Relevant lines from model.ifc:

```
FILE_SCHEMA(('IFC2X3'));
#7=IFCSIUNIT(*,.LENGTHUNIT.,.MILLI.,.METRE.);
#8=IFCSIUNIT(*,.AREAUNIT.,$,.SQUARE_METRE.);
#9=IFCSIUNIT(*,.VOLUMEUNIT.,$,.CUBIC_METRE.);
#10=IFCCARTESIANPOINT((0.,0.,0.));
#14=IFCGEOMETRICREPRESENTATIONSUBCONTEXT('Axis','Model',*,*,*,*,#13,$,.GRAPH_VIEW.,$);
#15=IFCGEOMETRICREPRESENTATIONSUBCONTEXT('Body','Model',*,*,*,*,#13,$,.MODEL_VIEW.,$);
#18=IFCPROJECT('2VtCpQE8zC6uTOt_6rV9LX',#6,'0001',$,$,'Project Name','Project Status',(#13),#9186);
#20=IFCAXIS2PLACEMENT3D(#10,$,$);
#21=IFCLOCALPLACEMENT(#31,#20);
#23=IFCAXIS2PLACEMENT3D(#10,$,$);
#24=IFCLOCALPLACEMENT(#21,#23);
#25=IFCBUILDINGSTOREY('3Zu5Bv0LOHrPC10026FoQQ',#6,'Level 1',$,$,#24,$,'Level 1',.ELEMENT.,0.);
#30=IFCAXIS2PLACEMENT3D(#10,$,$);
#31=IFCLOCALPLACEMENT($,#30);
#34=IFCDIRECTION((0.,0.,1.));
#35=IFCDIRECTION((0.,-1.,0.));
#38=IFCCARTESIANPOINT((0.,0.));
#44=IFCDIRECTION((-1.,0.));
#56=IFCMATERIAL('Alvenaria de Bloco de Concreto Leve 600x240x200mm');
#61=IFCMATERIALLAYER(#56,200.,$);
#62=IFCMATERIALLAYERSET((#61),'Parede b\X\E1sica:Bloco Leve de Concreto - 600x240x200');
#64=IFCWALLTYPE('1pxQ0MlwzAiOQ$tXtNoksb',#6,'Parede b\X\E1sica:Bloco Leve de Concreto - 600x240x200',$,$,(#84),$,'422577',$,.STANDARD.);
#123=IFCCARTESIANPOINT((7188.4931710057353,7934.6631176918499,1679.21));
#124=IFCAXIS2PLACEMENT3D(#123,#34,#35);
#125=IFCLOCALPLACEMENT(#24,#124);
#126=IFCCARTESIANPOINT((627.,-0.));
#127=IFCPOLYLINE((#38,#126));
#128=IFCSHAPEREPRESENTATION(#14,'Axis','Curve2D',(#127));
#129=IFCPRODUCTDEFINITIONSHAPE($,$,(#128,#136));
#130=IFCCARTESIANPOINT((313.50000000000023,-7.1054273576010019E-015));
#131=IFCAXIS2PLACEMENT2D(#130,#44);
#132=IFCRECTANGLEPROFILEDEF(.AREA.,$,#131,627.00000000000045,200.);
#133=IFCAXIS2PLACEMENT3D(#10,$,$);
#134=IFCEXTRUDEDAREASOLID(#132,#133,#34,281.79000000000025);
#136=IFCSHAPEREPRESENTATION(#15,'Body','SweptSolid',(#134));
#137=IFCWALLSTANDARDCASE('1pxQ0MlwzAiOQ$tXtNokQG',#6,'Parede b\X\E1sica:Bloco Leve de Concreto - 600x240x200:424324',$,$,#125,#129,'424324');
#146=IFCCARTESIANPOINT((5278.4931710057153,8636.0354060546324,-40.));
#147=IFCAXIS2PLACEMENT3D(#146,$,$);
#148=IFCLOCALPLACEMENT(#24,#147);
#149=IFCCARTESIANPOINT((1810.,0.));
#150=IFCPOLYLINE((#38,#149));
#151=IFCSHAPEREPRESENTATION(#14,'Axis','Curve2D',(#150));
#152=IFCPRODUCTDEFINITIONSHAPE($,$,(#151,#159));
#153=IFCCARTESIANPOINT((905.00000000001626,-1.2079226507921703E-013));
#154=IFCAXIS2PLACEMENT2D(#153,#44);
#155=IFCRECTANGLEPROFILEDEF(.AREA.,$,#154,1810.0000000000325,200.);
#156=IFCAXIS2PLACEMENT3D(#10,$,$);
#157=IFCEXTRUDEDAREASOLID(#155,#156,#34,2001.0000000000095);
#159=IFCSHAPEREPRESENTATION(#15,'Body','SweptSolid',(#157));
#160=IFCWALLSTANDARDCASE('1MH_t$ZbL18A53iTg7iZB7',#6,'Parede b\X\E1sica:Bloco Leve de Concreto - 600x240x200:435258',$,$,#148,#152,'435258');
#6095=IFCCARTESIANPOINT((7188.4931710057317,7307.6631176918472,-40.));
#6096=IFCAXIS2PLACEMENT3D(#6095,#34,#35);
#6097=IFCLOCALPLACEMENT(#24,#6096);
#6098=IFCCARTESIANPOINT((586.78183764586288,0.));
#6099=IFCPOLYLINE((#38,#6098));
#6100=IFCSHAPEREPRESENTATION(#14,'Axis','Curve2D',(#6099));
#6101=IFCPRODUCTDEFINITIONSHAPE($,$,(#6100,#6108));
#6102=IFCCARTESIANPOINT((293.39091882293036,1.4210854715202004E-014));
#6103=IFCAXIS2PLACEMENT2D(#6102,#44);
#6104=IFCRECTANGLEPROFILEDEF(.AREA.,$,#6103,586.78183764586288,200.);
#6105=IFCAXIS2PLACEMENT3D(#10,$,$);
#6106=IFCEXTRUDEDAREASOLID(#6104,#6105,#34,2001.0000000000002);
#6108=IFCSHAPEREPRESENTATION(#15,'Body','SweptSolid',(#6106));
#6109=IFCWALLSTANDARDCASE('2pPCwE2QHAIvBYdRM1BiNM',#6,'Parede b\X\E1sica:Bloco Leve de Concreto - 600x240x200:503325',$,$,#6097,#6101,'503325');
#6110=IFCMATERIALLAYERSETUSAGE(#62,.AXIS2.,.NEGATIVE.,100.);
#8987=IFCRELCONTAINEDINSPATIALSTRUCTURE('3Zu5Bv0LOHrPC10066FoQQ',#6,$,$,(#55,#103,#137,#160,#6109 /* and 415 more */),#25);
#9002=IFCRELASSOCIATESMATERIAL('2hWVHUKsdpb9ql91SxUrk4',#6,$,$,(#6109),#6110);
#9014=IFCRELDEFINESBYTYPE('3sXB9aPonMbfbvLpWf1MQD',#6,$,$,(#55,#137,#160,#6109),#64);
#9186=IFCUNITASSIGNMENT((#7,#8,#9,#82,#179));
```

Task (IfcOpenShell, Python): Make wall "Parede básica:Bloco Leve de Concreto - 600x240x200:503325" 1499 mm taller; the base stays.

```python
import ifcopenshell
import ifcopenshell.geom
import ifcopenshell.util.representation
import ifcopenshell.util.shape
import ifcopenshell.util.unit

model = ifcopenshell.open("model.ifc")
unit_scale = ifcopenshell.util.unit.calculate_unit_scale(model)
settings = ifcopenshell.geom.settings()


def volume(element):
    """Net volume in cubic metres, openings subtracted."""
    shape = ifcopenshell.geom.create_shape(settings, element)
    return ifcopenshell.util.shape.get_volume(shape.geometry)


wall = model.by_id(6109)
before = volume(wall)

body = ifcopenshell.util.representation.get_representation(wall, "Model", "Body")
solid = body.Items[0]
old_height = solid.Depth
solid.Depth += 1.499 / unit_scale
after = volume(wall)

print(f"height {old_height:g} -> {solid.Depth:g}, volume {before:.3f} -> {after:.3f} m3")

model.write("model_edited.ifc")
```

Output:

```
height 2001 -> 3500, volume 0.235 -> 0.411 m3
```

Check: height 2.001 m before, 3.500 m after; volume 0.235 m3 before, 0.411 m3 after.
